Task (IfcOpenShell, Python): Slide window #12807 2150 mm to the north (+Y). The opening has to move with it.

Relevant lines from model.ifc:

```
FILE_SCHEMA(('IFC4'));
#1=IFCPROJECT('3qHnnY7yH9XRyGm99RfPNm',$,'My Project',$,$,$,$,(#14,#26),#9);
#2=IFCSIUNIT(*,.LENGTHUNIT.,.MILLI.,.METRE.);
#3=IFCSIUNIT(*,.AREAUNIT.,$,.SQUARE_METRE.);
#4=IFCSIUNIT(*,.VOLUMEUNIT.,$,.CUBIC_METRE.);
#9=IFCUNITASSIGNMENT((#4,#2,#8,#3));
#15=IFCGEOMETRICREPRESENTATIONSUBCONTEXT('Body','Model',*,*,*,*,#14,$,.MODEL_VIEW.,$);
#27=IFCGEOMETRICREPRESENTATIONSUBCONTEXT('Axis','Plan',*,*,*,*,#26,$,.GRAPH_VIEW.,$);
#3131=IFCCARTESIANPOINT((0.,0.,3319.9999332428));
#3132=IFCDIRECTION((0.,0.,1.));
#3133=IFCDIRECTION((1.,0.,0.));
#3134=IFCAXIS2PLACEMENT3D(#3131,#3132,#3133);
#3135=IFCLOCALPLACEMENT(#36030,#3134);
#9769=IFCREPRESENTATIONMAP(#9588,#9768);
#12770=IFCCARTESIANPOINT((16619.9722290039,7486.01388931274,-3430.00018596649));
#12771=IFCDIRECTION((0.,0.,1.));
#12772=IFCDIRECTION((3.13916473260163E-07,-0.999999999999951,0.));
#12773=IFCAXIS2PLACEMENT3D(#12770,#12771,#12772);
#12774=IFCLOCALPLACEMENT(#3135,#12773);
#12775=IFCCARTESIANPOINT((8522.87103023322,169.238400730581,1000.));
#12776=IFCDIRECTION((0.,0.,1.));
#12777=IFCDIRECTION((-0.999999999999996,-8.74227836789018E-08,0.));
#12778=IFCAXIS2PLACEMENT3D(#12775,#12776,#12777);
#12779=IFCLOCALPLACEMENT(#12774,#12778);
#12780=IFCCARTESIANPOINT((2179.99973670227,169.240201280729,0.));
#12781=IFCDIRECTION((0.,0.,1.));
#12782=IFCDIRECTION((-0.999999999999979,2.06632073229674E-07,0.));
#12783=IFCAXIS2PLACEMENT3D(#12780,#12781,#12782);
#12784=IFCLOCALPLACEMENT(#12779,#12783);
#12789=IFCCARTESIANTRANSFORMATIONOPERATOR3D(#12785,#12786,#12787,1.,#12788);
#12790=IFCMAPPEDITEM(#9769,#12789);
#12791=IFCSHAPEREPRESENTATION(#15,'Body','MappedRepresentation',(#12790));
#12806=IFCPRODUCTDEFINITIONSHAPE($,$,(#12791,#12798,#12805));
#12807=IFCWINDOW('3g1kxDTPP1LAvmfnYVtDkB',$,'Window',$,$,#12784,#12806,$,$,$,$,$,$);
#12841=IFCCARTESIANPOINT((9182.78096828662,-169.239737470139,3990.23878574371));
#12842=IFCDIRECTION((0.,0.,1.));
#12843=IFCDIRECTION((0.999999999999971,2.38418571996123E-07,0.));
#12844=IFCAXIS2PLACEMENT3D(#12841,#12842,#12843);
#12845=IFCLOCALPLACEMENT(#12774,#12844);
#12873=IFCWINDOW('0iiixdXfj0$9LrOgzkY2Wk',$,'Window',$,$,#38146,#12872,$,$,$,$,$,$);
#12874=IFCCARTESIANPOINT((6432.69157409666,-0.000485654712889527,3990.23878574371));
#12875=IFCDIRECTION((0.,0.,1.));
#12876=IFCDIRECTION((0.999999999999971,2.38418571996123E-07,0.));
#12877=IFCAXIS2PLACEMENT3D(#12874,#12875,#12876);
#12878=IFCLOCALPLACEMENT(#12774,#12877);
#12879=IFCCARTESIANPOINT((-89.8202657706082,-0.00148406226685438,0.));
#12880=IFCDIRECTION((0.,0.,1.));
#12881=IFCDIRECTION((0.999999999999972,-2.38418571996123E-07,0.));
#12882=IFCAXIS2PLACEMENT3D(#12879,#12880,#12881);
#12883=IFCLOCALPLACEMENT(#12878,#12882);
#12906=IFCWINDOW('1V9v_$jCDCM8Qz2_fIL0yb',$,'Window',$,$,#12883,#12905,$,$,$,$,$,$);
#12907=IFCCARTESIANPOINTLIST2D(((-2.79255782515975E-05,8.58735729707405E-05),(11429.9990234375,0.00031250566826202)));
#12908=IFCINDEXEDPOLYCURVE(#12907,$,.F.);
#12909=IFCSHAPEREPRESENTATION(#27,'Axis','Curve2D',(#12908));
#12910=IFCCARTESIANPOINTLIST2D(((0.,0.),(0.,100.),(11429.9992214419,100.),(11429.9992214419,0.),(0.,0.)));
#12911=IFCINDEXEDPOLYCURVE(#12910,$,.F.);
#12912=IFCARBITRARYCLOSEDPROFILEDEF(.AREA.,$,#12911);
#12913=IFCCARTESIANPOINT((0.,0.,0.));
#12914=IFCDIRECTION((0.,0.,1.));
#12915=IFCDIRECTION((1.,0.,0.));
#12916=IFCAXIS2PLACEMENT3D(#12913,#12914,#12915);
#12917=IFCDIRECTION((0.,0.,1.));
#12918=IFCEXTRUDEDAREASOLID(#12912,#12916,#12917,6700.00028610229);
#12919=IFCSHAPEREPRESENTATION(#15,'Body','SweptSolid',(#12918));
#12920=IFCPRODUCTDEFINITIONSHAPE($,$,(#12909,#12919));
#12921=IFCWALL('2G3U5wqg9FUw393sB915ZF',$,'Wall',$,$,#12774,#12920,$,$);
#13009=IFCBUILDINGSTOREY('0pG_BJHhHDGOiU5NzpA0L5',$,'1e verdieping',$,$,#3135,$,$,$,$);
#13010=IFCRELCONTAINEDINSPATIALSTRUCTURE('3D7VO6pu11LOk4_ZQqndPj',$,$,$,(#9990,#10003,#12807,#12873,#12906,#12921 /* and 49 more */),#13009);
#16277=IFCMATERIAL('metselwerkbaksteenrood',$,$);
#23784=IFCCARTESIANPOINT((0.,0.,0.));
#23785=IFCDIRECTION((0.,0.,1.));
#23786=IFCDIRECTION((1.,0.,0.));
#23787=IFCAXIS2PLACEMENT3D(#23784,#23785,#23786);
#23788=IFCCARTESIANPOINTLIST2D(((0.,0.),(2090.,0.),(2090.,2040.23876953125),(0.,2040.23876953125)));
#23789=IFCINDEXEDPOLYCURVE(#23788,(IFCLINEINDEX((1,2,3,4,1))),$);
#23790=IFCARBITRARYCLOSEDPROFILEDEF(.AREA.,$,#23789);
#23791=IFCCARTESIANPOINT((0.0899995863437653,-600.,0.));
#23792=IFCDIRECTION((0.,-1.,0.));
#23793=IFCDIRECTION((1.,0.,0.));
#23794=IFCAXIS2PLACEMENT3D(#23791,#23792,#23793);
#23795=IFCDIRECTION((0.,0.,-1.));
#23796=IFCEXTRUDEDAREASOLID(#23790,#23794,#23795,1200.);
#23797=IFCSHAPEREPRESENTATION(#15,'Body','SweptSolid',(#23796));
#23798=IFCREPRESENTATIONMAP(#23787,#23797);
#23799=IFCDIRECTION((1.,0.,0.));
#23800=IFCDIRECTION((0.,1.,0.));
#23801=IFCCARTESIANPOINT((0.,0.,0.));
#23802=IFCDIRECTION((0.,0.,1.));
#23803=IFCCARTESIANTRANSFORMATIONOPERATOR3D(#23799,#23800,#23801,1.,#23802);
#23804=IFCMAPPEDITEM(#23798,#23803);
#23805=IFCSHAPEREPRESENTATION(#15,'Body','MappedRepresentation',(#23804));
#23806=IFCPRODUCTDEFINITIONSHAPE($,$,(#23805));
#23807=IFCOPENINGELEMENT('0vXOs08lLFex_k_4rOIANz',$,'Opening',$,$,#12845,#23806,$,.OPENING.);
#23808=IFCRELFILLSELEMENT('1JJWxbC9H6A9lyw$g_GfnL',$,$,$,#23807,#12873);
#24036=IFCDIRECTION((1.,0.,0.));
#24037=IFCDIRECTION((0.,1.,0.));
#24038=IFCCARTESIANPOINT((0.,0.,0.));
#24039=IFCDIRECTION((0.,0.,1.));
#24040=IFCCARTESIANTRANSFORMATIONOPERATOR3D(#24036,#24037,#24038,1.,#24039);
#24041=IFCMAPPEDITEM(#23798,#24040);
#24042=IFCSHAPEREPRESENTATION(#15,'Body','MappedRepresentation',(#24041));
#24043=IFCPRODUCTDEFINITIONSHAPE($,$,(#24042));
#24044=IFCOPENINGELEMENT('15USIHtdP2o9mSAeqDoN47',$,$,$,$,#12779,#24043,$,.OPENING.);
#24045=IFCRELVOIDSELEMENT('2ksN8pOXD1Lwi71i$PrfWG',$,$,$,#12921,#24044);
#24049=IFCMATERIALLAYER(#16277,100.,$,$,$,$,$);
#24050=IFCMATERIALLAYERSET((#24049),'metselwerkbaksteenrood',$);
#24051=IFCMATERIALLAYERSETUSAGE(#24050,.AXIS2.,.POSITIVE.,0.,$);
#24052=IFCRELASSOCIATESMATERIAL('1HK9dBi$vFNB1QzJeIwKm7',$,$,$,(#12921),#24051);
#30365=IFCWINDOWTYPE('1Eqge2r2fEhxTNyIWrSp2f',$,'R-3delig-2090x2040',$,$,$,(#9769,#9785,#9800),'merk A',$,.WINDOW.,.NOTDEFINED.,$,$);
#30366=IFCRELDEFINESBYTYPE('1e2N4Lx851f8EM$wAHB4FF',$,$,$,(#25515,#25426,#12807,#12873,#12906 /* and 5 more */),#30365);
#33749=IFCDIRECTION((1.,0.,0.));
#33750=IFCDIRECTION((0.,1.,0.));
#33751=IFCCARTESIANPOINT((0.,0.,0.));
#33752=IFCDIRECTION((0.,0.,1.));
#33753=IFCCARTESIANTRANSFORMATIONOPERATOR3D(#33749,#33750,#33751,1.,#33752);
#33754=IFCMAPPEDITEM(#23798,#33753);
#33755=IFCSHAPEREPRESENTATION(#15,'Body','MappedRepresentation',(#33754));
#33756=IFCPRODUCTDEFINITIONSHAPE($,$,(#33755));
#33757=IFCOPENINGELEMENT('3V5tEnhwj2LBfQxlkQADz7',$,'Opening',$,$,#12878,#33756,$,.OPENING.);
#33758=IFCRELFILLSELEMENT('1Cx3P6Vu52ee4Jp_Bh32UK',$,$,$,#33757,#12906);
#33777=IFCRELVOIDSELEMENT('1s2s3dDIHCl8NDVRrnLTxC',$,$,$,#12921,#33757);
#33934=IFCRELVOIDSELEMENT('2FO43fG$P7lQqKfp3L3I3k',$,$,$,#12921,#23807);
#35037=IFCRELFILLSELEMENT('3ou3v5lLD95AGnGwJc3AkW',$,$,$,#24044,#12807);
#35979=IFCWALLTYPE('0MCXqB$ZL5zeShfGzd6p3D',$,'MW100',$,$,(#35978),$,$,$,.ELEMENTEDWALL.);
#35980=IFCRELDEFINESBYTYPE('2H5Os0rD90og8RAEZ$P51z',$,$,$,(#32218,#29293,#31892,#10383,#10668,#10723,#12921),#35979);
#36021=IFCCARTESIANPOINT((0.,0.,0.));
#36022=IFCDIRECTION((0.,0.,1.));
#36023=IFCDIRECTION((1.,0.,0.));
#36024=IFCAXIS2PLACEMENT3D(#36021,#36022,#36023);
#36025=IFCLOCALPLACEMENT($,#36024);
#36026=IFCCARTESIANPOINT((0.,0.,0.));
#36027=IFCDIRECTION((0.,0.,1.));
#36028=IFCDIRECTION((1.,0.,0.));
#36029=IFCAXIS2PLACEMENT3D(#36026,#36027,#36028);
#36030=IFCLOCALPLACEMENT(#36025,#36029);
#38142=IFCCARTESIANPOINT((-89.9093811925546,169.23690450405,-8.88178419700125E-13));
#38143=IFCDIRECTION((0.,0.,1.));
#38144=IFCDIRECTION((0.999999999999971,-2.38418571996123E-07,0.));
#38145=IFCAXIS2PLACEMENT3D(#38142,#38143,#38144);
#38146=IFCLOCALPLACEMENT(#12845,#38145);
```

```python
import ifcopenshell
import ifcopenshell.api.geometry
import ifcopenshell.util.placement
import ifcopenshell.util.unit

model = ifcopenshell.open("model.ifc")
unit_scale = ifcopenshell.util.unit.calculate_unit_scale(model)

window = model.by_guid("3g1kxDTPP1LAvmfnYVtDkB")
opening = window.FillsVoids[0].RelatingOpeningElement
wall = opening.VoidsElements[0].RelatingBuildingElement

wall_matrix = ifcopenshell.util.placement.get_local_placement(wall.ObjectPlacement)
shift = wall_matrix[:3, 0] * -2.15 / unit_scale
before = ifcopenshell.util.placement.get_local_placement(window.ObjectPlacement)[:3, 3].copy()

# The window is placed relative to its opening, so it follows when the opening moves.
matrix = ifcopenshell.util.placement.get_local_placement(opening.ObjectPlacement)
matrix[:3, 3] += shift
ifcopenshell.api.geometry.edit_object_placement(
    model, product=opening, matrix=matrix, is_si=False, should_transform_children=True
)

after = ifcopenshell.util.placement.get_local_placement(window.ObjectPlacement)[:3, 3]
print("window moved by", (after - before).round(3) + 0.0)

model.write("model_edited.ifc")
```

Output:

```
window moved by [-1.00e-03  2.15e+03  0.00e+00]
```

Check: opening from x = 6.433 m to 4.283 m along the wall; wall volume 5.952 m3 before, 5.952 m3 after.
